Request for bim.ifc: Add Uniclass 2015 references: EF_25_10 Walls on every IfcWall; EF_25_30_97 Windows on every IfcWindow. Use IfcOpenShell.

First a look at what the model holds.

```python
import ifcopenshell

model = ifcopenshell.open("bim.ifc")
print(model.schema)
print("classifications:", [c.Name for c in model.by_type("IfcClassification")])
for ifc_class in ("IfcDoor", "IfcRoof", "IfcStair", "IfcWall", "IfcWindow"):
    print(ifc_class, len(model.by_type(ifc_class)))
```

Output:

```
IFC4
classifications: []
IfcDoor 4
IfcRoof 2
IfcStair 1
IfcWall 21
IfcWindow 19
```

```python
import ifcopenshell
import ifcopenshell.api.classification

model = ifcopenshell.open("bim.ifc")

system = ifcopenshell.api.classification.add_classification(model, classification="Uniclass 2015")

codes = {
    "IfcWall": ("EF_25_10", "Walls"),
    "IfcWindow": ("EF_25_30_97", "Windows"),
}
for ifc_class, (code, name) in codes.items():
    products = model.by_type(ifc_class)
    ifcopenshell.api.classification.add_reference(
        model, products=products, classification=system, identification=code, name=name
    )
    print(code, len(products))

model.write("bim_updated.ifc")
```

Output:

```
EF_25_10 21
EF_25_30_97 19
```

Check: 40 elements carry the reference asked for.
